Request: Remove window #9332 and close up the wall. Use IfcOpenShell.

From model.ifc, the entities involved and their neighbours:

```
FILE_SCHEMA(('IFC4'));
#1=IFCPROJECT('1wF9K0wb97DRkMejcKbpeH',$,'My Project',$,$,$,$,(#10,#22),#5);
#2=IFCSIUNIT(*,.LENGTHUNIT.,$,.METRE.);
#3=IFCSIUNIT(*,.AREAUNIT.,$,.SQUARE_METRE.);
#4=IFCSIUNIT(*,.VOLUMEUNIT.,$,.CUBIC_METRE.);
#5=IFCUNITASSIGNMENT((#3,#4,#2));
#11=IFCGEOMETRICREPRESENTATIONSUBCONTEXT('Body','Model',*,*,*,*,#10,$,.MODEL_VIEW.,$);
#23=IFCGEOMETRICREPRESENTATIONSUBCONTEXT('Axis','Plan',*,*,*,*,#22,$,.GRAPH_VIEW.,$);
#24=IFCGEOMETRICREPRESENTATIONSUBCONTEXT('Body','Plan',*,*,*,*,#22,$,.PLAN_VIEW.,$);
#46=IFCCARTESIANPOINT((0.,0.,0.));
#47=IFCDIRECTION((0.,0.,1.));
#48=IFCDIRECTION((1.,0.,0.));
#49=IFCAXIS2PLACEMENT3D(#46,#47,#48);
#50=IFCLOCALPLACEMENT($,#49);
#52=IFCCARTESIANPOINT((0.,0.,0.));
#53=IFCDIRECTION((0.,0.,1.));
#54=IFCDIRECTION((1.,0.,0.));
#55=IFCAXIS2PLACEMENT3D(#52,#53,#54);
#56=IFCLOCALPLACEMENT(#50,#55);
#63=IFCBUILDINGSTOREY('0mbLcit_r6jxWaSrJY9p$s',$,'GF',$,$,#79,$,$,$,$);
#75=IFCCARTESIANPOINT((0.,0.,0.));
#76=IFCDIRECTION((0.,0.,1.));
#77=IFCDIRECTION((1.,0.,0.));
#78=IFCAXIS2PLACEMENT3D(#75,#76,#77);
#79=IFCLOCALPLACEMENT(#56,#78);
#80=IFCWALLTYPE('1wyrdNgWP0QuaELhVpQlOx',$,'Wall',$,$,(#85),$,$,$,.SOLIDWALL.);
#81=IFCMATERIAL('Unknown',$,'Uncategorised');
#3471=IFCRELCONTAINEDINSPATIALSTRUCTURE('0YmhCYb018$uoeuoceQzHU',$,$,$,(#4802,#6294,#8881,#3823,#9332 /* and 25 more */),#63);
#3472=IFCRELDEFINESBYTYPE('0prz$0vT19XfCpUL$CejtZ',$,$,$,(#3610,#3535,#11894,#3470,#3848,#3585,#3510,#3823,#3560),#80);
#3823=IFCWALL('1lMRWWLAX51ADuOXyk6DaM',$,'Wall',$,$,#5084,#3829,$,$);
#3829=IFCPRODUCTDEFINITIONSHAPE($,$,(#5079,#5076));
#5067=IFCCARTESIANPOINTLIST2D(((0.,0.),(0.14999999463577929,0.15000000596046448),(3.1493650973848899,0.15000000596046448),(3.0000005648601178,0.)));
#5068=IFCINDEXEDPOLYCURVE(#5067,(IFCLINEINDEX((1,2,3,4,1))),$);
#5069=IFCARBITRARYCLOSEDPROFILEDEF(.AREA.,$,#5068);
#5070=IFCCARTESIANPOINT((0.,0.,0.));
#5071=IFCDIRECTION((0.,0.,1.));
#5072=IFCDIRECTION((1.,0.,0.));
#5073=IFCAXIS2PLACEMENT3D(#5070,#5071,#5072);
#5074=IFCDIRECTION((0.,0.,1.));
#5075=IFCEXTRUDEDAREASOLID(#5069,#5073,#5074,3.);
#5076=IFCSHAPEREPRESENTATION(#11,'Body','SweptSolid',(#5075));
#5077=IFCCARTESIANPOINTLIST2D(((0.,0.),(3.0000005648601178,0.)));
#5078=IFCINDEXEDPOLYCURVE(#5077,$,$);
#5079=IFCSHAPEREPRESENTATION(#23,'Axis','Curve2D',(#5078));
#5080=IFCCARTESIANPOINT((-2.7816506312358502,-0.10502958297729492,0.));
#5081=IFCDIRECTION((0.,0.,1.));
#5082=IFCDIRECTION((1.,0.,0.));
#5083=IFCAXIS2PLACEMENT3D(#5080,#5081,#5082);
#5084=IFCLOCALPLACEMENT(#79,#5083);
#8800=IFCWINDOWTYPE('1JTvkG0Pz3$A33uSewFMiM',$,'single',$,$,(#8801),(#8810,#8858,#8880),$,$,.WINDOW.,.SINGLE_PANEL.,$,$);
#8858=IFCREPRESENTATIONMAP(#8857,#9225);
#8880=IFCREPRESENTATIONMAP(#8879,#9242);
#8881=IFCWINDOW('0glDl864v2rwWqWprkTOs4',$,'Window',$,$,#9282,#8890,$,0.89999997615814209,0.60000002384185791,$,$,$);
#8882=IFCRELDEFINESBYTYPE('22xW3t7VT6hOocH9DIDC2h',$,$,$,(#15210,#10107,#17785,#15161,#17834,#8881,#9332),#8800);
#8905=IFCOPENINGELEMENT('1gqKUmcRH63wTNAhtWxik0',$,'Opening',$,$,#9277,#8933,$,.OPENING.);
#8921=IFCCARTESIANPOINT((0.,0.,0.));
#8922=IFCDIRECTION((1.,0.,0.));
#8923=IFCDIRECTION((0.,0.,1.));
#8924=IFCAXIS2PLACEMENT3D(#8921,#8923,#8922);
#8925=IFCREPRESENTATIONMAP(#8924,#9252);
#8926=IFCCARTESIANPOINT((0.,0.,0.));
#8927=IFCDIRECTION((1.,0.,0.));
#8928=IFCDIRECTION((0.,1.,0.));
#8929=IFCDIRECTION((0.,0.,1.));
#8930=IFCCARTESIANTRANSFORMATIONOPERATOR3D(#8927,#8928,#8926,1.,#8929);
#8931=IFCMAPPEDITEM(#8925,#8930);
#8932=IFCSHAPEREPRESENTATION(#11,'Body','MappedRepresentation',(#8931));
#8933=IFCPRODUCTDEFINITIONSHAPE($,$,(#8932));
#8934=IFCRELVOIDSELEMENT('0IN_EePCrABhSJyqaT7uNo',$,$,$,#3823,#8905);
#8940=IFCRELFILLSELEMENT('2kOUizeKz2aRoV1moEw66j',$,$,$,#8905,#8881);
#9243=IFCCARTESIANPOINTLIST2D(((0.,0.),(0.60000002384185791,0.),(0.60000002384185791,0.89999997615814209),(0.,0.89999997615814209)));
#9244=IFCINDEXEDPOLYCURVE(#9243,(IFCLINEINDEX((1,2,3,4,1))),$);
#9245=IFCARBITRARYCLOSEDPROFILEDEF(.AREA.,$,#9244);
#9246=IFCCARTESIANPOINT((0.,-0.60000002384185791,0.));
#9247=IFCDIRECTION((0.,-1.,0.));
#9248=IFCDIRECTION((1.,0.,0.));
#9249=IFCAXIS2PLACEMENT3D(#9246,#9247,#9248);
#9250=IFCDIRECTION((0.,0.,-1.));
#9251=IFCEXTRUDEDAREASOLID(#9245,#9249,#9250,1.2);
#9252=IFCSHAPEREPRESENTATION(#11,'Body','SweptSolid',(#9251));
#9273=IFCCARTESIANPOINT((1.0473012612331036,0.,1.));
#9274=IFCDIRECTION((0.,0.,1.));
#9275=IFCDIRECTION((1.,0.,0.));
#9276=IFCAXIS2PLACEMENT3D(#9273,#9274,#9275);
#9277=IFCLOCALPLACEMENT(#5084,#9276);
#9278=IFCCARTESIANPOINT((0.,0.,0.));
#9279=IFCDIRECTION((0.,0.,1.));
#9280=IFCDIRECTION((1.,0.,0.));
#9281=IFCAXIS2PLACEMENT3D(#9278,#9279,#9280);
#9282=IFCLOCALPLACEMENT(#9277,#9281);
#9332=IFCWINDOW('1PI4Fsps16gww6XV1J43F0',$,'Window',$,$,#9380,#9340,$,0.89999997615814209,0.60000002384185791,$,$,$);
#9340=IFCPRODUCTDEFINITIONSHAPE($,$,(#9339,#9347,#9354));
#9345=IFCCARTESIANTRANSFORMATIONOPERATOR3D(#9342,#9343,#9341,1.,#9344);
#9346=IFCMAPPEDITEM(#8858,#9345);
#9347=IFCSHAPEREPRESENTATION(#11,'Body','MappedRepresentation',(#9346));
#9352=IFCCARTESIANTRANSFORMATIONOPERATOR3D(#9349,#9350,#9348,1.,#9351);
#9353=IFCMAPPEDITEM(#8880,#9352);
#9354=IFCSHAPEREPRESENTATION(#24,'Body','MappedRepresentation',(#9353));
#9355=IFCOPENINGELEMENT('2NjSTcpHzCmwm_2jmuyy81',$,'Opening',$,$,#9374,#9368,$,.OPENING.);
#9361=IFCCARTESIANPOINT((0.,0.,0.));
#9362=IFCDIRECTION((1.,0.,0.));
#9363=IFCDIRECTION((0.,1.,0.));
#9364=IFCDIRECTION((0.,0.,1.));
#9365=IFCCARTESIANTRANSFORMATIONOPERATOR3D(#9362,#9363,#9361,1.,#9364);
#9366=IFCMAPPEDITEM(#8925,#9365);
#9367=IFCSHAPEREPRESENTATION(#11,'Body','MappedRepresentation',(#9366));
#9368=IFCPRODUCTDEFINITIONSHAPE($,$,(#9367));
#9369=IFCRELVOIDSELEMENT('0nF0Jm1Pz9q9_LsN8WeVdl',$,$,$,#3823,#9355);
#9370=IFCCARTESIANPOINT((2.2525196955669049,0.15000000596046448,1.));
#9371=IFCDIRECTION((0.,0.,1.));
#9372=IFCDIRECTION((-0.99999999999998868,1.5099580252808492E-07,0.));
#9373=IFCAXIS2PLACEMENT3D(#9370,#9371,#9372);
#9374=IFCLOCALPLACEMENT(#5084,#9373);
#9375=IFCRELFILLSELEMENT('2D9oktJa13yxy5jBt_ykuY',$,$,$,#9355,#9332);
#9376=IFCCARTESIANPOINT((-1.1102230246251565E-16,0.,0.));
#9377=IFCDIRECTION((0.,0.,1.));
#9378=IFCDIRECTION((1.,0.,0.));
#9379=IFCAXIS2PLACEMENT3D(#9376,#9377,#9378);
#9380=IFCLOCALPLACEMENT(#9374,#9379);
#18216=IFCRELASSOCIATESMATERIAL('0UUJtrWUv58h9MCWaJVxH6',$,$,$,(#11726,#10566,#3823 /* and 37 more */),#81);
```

```python
import ifcopenshell
import ifcopenshell.api.feature
import ifcopenshell.api.root
import ifcopenshell.geom
import ifcopenshell.util.shape

model = ifcopenshell.open("model.ifc")
settings = ifcopenshell.geom.settings()


def volume(element):
    """Net volume in cubic metres, openings subtracted."""
    shape = ifcopenshell.geom.create_shape(settings, element)
    return ifcopenshell.util.shape.get_volume(shape.geometry)


window = model.by_guid("1PI4Fsps16gww6XV1J43F0")
opening = window.FillsVoids[0].RelatingOpeningElement
wall = opening.VoidsElements[0].RelatingBuildingElement
before = volume(wall)

ifcopenshell.api.root.remove_product(model, product=window)
ifcopenshell.api.feature.remove_feature(model, feature=opening)

after = volume(wall)

print(f"wall volume {before:.3f} -> {after:.3f} m3")

model.write("model_v2.ifc")
```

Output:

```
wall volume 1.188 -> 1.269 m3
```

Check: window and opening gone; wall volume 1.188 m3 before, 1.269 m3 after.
